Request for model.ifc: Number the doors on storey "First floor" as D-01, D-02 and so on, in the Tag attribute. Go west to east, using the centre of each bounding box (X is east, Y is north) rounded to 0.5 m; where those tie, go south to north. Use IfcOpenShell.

First a look at what the model holds.

```python
import ifcopenshell
import ifcopenshell.util.element
import ifcopenshell.util.placement

model = ifcopenshell.open("model.ifc")
print(model.schema)
storey = next(s for s in model.by_type("IfcBuildingStorey") if s.Name == "First floor")
doors = [e for e in ifcopenshell.util.element.get_decomposition(storey) if e.is_a("IfcDoor")]
for e in sorted(doors, key=lambda e: e.id()):
    origin = ifcopenshell.util.placement.get_local_placement(e.ObjectPlacement)[:3, 3]
    print(e.id(), e.Tag, e.Name, origin.round(2) + 0.0, sep=" | ")
```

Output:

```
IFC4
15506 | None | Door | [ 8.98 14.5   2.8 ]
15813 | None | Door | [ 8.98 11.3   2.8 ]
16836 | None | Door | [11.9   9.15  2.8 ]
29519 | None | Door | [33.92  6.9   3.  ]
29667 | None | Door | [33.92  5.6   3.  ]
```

```python
import ifcopenshell
import ifcopenshell.geom
import ifcopenshell.util.element
import ifcopenshell.util.shape

model = ifcopenshell.open("model.ifc")
settings = ifcopenshell.geom.settings()
settings.set("use-world-coords", True)


def centre(element):
    shape = ifcopenshell.geom.create_shape(settings, element)
    return ifcopenshell.util.shape.get_bbox_centroid(shape.geometry)


storey = next(s for s in model.by_type("IfcBuildingStorey") if s.Name == "First floor")
doors = [e for e in ifcopenshell.util.element.get_decomposition(storey) if e.is_a("IfcDoor")]

# Insertion points can sit at a corner or the storey origin, so sort by the geometry (in metres).
centres = {e: centre(e) for e in doors}
doors.sort(key=lambda e: (round(centres[e][0] / 0.5), centres[e][1]))

for i, e in enumerate(doors, start=1):
    number = f"D-{i:02d}"
    e.Tag = number
    print(e.id(), number)

model.write("model_edited.ifc")
```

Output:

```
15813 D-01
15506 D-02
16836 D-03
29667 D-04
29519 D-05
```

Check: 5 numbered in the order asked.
